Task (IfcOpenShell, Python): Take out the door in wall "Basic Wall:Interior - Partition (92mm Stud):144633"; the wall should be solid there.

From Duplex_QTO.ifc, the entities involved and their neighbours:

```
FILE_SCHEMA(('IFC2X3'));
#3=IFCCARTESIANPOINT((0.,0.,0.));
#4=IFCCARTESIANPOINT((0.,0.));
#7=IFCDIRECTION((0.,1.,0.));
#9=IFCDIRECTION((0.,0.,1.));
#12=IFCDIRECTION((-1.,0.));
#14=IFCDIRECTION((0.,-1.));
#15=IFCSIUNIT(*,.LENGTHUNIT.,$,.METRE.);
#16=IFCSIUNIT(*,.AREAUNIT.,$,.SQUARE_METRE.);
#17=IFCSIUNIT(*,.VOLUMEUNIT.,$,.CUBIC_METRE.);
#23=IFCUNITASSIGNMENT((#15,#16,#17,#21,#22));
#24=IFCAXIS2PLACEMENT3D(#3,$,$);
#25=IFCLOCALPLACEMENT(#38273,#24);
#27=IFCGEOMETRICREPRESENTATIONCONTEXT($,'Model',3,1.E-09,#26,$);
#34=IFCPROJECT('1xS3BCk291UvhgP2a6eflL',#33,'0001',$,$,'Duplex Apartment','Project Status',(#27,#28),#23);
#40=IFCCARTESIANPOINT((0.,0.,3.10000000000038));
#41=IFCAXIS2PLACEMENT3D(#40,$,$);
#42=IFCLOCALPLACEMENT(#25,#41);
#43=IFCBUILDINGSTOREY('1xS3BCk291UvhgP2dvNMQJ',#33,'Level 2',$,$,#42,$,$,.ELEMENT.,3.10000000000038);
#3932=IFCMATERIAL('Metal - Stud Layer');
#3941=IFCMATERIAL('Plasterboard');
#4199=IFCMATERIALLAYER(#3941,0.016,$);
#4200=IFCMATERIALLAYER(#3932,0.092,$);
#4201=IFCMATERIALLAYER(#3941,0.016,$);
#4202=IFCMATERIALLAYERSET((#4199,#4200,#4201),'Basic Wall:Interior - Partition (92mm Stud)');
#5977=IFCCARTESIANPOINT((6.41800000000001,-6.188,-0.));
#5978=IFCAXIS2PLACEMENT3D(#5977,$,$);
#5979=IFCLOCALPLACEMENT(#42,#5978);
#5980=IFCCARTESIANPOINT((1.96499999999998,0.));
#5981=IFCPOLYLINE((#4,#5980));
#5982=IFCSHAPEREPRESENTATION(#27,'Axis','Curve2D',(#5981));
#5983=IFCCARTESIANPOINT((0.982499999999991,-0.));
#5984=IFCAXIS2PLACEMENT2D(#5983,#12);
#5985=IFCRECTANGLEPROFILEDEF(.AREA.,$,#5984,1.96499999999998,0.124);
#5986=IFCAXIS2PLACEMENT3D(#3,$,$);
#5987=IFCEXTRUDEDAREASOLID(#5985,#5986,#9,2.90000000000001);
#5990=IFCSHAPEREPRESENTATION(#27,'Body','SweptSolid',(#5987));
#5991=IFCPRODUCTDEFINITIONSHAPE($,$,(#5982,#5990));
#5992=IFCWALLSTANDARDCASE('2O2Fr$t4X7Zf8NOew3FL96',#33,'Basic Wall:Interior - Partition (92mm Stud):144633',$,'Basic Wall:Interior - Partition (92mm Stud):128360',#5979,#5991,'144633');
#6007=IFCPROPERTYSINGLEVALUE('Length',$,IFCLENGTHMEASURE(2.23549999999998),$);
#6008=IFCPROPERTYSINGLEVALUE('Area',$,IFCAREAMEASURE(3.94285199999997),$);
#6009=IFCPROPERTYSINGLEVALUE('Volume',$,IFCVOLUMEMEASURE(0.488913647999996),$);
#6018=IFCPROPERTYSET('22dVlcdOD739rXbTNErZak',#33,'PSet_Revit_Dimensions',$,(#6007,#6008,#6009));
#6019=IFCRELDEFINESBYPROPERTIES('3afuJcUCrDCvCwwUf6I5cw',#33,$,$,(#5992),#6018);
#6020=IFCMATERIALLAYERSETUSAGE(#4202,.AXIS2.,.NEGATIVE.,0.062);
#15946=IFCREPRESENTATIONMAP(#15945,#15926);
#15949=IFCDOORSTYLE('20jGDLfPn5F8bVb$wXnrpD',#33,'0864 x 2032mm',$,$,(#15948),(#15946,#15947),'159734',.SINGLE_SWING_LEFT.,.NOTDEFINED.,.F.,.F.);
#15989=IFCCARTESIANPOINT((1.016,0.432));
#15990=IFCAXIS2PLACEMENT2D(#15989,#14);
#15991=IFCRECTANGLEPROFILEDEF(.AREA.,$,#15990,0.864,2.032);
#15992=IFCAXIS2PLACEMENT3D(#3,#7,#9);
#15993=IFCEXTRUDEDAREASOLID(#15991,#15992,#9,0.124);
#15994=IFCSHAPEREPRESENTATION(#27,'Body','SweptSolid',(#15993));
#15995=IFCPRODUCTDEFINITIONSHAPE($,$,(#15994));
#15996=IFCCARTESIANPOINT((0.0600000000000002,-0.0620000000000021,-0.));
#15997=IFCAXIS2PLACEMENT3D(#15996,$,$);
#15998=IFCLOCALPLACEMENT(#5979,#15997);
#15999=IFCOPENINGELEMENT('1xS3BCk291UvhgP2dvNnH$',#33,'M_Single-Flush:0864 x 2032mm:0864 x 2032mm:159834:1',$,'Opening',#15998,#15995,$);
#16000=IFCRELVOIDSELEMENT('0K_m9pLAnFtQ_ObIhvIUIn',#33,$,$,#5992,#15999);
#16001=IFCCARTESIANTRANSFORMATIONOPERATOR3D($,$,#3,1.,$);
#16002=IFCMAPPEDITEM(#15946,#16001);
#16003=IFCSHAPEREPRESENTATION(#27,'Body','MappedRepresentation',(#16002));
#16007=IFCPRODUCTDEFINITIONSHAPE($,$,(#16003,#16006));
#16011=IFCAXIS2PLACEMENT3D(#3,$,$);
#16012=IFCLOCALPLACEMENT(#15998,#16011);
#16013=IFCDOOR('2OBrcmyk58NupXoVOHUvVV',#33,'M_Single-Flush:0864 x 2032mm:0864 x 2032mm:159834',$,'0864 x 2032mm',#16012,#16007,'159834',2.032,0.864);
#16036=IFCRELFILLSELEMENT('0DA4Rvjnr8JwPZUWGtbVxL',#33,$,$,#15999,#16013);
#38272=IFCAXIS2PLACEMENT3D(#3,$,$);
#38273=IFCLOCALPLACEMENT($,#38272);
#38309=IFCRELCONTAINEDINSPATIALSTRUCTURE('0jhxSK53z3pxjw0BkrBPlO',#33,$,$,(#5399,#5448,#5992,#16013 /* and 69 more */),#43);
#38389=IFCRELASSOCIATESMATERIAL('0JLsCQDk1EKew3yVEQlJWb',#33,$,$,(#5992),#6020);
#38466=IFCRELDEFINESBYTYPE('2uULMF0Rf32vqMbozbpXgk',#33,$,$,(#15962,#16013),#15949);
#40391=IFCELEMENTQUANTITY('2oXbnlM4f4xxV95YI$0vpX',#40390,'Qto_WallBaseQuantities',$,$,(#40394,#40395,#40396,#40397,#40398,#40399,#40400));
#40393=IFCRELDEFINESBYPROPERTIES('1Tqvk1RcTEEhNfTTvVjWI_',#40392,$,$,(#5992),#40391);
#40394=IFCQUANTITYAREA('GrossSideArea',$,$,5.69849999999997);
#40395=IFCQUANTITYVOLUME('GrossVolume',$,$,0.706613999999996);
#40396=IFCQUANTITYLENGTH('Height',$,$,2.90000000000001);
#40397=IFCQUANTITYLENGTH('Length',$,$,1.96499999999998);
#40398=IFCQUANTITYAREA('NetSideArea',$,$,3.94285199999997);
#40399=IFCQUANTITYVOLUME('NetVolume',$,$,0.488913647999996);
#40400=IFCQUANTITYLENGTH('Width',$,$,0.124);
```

```python
import ifcopenshell
import ifcopenshell.api.feature
import ifcopenshell.api.pset
import ifcopenshell.api.root
import ifcopenshell.geom
import ifcopenshell.util.element
import ifcopenshell.util.shape
import ifcopenshell.util.unit

model = ifcopenshell.open("Duplex_QTO.ifc")
area_scale = ifcopenshell.util.unit.calculate_unit_scale(model, "AREAUNIT")
volume_scale = ifcopenshell.util.unit.calculate_unit_scale(model, "VOLUMEUNIT")
settings = ifcopenshell.geom.settings()


def volume(element):
    """Net volume in cubic metres, openings subtracted."""
    shape = ifcopenshell.geom.create_shape(settings, element)
    return ifcopenshell.util.shape.get_volume(shape.geometry)


door = model.by_guid("2OBrcmyk58NupXoVOHUvVV")
opening = door.FillsVoids[0].RelatingOpeningElement
wall = opening.VoidsElements[0].RelatingBuildingElement
before = volume(wall)

ifcopenshell.api.root.remove_product(model, product=door)
ifcopenshell.api.feature.remove_feature(model, feature=opening)

after = volume(wall)
thickness = 0.124  # wall thickness in metres

# Update the wall's stored quantities.
pset = model.by_id(ifcopenshell.util.element.get_pset(wall, "PSet_Revit_Dimensions", should_inherit=False)["id"])
ifcopenshell.api.pset.edit_pset(model, pset=pset, properties={
    "Area": model.create_entity("IfcAreaMeasure", after / thickness / area_scale),
    "Volume": model.create_entity("IfcVolumeMeasure", after / volume_scale),
})
qto = model.by_id(ifcopenshell.util.element.get_pset(wall, "Qto_WallBaseQuantities", should_inherit=False)["id"])
ifcopenshell.api.pset.edit_qto(model, qto=qto, properties={
    "NetSideArea": after / thickness / area_scale,
    "NetVolume": after / volume_scale,
})

print(f"wall volume {before:.3f} -> {after:.3f} m3")

model.write("Duplex_QTO_updated.ifc")
```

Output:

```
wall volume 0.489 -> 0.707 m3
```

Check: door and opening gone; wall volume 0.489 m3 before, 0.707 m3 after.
